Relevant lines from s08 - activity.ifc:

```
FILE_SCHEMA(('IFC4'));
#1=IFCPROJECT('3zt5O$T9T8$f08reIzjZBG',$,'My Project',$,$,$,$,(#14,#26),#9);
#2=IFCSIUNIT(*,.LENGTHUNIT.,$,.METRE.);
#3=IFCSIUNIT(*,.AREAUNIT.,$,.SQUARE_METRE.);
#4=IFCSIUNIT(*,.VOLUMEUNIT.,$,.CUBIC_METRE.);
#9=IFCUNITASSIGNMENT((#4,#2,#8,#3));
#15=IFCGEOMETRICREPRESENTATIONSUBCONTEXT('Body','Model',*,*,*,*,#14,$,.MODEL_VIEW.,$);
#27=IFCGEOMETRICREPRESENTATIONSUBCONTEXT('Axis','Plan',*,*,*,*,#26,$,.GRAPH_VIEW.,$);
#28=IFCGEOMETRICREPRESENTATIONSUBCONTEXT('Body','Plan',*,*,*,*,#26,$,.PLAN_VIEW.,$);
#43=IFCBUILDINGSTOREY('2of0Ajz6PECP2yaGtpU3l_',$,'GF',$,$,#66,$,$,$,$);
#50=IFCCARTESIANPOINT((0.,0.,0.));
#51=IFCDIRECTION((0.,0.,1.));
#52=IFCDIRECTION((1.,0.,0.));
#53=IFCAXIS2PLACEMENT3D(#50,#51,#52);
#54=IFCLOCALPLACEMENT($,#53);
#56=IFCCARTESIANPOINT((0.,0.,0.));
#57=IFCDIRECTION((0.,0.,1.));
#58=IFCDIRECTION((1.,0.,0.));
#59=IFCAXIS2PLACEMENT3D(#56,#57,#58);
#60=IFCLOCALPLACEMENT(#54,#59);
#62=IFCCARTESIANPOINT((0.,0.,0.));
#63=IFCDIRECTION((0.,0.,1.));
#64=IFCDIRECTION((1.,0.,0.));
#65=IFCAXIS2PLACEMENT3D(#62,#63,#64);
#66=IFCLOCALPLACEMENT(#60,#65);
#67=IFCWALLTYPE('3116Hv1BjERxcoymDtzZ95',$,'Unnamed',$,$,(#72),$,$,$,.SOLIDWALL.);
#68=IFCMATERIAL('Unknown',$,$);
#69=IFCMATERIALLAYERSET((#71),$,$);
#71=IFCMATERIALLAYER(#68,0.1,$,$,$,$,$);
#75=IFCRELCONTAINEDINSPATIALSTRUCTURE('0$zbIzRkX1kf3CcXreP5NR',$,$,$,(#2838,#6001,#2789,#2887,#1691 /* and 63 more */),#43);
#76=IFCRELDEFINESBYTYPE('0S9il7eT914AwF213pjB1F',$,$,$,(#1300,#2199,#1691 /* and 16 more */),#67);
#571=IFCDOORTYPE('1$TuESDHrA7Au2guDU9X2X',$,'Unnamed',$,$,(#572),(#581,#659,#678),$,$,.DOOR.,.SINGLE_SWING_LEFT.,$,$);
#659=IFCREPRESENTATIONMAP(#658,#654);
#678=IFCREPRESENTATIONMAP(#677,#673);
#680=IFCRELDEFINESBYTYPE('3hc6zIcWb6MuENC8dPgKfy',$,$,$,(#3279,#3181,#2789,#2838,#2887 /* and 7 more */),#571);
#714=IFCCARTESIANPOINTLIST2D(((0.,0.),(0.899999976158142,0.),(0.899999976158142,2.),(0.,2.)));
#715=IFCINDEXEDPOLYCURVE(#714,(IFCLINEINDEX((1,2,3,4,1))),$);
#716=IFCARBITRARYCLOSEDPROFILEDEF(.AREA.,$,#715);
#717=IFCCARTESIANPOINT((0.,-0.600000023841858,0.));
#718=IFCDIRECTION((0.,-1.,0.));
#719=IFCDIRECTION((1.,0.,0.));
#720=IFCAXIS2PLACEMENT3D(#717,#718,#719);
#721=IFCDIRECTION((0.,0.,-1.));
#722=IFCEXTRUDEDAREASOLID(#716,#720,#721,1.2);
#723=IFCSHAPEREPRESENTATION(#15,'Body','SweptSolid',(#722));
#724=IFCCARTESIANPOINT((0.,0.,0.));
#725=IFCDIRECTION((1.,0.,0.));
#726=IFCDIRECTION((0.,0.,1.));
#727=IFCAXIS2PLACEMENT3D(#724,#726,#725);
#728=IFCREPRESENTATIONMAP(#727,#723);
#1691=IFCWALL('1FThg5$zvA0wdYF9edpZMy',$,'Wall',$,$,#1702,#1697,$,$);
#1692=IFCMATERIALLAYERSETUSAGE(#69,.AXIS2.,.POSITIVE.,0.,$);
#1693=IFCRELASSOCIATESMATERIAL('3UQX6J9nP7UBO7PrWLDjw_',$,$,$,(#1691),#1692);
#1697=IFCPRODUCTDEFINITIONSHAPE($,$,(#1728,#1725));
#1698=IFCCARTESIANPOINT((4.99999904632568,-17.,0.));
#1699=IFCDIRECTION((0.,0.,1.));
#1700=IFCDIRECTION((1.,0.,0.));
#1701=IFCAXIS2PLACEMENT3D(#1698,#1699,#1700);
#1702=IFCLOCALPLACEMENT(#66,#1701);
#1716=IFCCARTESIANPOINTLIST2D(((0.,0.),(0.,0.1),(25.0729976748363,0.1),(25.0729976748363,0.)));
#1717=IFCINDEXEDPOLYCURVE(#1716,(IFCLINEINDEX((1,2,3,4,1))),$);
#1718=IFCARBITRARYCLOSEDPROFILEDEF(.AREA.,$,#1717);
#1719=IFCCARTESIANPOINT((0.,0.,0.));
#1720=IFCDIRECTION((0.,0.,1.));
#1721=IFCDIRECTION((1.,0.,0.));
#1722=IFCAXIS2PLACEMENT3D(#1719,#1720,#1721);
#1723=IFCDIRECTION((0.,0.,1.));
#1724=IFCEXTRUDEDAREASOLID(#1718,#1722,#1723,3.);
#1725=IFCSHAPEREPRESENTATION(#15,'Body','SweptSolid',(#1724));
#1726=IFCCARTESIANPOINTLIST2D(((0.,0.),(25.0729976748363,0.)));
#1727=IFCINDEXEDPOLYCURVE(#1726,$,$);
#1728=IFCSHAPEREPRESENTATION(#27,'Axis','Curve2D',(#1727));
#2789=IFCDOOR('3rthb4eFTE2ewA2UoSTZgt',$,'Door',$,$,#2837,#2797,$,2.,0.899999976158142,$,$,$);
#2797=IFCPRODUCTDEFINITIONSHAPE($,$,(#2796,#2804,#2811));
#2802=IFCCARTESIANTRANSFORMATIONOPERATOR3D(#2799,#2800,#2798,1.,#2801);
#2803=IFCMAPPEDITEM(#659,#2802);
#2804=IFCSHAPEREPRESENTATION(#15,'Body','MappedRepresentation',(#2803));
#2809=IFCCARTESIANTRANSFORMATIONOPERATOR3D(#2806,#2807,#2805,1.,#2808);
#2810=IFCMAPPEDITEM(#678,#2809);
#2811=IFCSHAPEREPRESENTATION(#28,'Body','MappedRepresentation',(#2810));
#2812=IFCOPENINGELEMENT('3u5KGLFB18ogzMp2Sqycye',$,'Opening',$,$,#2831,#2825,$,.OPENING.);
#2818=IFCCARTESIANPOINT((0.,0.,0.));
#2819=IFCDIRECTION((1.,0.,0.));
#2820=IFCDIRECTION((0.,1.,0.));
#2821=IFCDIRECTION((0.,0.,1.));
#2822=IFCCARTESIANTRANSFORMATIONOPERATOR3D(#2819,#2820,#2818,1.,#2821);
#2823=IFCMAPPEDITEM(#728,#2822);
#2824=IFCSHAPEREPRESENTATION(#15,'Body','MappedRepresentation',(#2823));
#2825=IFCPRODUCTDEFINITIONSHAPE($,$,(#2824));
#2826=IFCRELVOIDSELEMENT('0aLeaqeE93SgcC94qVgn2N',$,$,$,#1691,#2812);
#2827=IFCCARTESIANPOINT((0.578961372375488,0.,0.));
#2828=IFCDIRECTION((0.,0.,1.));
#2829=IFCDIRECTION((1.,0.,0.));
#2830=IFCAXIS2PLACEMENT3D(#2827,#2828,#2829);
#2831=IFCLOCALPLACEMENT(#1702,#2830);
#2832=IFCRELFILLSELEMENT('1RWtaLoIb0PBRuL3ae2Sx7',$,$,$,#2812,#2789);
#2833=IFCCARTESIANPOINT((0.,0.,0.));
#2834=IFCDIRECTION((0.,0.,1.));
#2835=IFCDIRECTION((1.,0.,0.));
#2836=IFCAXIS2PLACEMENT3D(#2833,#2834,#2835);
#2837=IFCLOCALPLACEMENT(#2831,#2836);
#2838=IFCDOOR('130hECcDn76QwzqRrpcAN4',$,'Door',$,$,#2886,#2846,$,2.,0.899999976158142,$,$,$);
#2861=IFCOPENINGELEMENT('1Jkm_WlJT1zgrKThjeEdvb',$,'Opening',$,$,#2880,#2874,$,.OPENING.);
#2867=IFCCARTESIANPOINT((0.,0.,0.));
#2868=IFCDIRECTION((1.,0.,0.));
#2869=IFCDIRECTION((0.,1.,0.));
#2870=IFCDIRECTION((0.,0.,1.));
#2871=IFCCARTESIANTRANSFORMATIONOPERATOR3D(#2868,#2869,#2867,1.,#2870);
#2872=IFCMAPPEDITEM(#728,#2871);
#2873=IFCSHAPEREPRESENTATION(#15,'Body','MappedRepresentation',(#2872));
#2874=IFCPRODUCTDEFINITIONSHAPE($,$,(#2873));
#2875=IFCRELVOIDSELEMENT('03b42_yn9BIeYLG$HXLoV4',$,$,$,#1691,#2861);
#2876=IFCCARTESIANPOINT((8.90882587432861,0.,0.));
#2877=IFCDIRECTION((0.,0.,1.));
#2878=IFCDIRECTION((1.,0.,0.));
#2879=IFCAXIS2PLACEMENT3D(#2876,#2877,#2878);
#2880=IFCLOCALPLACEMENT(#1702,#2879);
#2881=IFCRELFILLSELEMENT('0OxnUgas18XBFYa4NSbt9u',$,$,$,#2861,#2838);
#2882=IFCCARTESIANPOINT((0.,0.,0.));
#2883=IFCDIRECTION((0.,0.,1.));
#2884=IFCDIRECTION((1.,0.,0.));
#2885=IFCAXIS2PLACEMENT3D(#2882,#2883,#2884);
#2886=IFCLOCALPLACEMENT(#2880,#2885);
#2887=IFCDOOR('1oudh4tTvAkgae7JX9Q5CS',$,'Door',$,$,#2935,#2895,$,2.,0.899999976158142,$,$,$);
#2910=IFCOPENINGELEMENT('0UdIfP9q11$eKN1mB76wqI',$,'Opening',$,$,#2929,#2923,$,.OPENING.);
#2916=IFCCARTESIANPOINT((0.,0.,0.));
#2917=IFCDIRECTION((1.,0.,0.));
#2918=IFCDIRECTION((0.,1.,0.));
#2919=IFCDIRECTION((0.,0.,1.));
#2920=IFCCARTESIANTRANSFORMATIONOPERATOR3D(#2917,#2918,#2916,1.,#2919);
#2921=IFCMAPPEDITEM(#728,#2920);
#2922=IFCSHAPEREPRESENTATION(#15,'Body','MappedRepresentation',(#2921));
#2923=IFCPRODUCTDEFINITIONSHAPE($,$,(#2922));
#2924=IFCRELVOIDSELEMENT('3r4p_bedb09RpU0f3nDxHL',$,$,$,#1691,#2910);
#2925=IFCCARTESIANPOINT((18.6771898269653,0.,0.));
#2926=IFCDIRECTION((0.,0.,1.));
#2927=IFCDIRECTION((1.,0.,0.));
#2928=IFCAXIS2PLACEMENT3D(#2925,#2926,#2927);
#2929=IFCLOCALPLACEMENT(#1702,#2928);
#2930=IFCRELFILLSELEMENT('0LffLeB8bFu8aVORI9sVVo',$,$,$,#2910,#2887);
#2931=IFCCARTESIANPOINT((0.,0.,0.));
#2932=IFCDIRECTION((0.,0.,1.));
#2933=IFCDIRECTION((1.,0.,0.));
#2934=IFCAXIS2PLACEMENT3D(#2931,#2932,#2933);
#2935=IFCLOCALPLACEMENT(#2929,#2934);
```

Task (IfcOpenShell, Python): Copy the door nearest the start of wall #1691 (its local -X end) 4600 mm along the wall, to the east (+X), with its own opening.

```python
import ifcopenshell
import ifcopenshell.api.feature
import ifcopenshell.api.geometry
import ifcopenshell.api.root
import ifcopenshell.geom
import ifcopenshell.util.element
import ifcopenshell.util.placement
import ifcopenshell.util.shape
import ifcopenshell.util.unit

model = ifcopenshell.open("s08 - activity.ifc")
unit_scale = ifcopenshell.util.unit.calculate_unit_scale(model)
settings = ifcopenshell.geom.settings()


def volume(element):
    """Net volume in cubic metres, openings subtracted."""
    shape = ifcopenshell.geom.create_shape(settings, element)
    return ifcopenshell.util.shape.get_volume(shape.geometry)


door = model.by_guid("3rthb4eFTE2ewA2UoSTZgt")
opening = door.FillsVoids[0].RelatingOpeningElement
wall = opening.VoidsElements[0].RelatingBuildingElement
before = volume(wall)
shift = ifcopenshell.util.placement.get_local_placement(wall.ObjectPlacement)[:3, 0] * 4.6 / unit_scale

# copy_class copies the void relationship, type, container and properties, but no geometry.
new_opening = ifcopenshell.api.root.copy_class(model, product=opening)
new_opening.Representation = ifcopenshell.util.element.copy_deep(
    model, opening.Representation, exclude=["IfcGeometricRepresentationContext", "IfcRepresentationMap"]
)
new_door = ifcopenshell.api.root.copy_class(model, product=door)
new_door.Representation = ifcopenshell.util.element.copy_deep(
    model, door.Representation, exclude=["IfcGeometricRepresentationContext", "IfcRepresentationMap"]
)
ifcopenshell.api.feature.add_filling(model, opening=new_opening, element=new_door)

for old, new in ((opening, new_opening), (door, new_door)):
    matrix = ifcopenshell.util.placement.get_local_placement(old.ObjectPlacement)
    matrix[:3, 3] += shift
    ifcopenshell.api.geometry.edit_object_placement(model, product=new, matrix=matrix, is_si=False)

after = volume(wall)

print(f"wall volume {before:.3f} -> {after:.3f} m3")

model.write("s08 - activity_rev.ifc")
```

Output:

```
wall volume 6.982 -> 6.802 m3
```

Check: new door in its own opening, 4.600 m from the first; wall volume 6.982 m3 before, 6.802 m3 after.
